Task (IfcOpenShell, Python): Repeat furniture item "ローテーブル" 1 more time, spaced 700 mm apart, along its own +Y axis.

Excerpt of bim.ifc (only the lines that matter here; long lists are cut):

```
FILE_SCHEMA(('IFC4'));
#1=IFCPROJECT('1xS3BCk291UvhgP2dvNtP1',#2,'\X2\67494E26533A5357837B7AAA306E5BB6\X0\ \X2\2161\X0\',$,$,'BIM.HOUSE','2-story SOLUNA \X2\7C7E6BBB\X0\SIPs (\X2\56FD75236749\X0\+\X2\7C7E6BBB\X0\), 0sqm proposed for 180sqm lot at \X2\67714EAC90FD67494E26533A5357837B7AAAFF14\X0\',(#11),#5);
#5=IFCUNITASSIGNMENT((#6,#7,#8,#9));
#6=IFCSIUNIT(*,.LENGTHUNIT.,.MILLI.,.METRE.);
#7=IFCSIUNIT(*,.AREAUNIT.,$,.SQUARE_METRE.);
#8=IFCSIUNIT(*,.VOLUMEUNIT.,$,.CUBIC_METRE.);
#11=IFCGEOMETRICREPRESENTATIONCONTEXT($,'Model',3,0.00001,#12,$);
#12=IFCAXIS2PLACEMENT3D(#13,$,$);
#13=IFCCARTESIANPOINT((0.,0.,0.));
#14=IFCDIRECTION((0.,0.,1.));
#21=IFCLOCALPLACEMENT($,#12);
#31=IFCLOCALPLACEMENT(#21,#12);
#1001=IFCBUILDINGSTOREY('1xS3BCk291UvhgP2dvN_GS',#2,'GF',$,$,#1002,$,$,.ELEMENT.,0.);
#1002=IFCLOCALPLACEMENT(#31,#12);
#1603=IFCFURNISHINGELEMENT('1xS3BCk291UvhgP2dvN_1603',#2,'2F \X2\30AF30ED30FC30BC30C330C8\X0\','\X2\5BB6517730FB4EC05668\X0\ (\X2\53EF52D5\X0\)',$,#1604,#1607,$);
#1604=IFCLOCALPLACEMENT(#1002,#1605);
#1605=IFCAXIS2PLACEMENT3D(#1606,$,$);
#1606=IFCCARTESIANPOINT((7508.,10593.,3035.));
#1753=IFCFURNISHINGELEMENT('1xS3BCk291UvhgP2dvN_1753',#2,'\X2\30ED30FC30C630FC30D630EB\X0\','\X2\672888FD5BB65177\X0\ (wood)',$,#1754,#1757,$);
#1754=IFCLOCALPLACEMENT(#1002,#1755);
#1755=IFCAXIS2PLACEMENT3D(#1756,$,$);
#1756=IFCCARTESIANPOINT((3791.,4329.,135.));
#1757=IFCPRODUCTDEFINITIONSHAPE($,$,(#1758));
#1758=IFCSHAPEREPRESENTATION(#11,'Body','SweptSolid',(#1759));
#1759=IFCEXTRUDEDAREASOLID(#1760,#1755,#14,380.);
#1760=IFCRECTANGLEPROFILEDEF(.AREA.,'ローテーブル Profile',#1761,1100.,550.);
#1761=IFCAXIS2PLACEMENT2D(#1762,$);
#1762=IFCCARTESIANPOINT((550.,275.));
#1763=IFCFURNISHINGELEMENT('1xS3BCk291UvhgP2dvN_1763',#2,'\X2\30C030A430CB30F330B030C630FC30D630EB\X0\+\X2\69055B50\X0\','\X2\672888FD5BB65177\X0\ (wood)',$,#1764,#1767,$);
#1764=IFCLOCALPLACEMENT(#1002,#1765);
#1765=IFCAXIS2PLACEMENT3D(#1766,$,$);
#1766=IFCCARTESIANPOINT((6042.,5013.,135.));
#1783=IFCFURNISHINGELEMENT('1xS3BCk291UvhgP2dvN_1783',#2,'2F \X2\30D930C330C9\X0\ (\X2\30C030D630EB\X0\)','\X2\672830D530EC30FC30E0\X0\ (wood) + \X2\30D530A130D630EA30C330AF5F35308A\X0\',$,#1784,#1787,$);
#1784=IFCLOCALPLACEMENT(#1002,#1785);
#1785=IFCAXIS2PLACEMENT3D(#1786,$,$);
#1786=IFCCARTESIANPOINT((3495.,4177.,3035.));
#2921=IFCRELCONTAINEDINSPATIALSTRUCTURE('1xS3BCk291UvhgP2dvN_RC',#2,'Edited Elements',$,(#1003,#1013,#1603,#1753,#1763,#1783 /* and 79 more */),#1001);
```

```python
import ifcopenshell
import ifcopenshell.api.geometry
import ifcopenshell.api.root
import ifcopenshell.util.element
import ifcopenshell.util.placement

model = ifcopenshell.open("bim.ifc")


def reuse_history(source, copy):
    """copy_class also copies each property set's owner history, people and application; keep the originals."""
    for rel in copy.IsDefinedBy:
        if rel.is_a("IfcRelDefinesByProperties") and (history := rel.RelatingPropertyDefinition.OwnerHistory):
            rel.RelatingPropertyDefinition.OwnerHistory = source.OwnerHistory
            ifcopenshell.util.element.remove_deep2(model, history)


source = model.by_id(1753)
base = ifcopenshell.util.placement.get_local_placement(source.ObjectPlacement)
step = base[:3, 1] * 700.0

for i in range(1, 2):
    copy = ifcopenshell.api.root.copy_class(model, product=source)
    copy.Representation = ifcopenshell.util.element.copy_deep(
        model, source.Representation, exclude=["IfcGeometricRepresentationContext", "IfcRepresentationMap"]
    )
    reuse_history(source, copy)
    matrix = base.copy()
    matrix[:3, 3] += i * step
    print("added at", matrix[:3, 3].round(3) + 0.0)
    ifcopenshell.api.geometry.edit_object_placement(model, product=copy, matrix=matrix, is_si=False)

model.write("bim_rev.ifc")
```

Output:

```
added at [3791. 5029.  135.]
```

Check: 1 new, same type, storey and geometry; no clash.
